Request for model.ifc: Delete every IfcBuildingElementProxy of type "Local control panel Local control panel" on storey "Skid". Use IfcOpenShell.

First a look at what the model holds.

```python
import ifcopenshell
import ifcopenshell.util.element

model = ifcopenshell.open("model.ifc")
print(model.schema)
storey = next(s for s in model.by_type("IfcBuildingStorey") if s.Name == "Skid")
proxies = [e for e in ifcopenshell.util.element.get_decomposition(storey) if e.is_a("IfcBuildingElementProxy")]
seen = {}
for e in proxies:
    element_type = ifcopenshell.util.element.get_type(e)
    name = element_type.Name if element_type not in (None, e) else None
    seen[name] = seen.get(name, 0) + 1
for name, count in sorted(seen.items(), key=str):
    print(count, "x", name)
```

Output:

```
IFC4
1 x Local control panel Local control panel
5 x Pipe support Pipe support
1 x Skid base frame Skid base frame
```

```python
import ifcopenshell
import ifcopenshell.api.root
import ifcopenshell.util.element

model = ifcopenshell.open("model.ifc")

storey = next(s for s in model.by_type("IfcBuildingStorey") if s.Name == "Skid")
proxies = [e for e in ifcopenshell.util.element.get_decomposition(storey) if e.is_a("IfcBuildingElementProxy")]
targets = [e for e in proxies if (t := ifcopenshell.util.element.get_type(e)) not in (None, e) and t.Name == "Local control panel Local control panel"]

for e in targets:
    ifcopenshell.api.root.remove_product(model, product=e)
print(len(targets), "removed")

model.write("model_rev.ifc")
```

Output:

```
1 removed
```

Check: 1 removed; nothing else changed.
